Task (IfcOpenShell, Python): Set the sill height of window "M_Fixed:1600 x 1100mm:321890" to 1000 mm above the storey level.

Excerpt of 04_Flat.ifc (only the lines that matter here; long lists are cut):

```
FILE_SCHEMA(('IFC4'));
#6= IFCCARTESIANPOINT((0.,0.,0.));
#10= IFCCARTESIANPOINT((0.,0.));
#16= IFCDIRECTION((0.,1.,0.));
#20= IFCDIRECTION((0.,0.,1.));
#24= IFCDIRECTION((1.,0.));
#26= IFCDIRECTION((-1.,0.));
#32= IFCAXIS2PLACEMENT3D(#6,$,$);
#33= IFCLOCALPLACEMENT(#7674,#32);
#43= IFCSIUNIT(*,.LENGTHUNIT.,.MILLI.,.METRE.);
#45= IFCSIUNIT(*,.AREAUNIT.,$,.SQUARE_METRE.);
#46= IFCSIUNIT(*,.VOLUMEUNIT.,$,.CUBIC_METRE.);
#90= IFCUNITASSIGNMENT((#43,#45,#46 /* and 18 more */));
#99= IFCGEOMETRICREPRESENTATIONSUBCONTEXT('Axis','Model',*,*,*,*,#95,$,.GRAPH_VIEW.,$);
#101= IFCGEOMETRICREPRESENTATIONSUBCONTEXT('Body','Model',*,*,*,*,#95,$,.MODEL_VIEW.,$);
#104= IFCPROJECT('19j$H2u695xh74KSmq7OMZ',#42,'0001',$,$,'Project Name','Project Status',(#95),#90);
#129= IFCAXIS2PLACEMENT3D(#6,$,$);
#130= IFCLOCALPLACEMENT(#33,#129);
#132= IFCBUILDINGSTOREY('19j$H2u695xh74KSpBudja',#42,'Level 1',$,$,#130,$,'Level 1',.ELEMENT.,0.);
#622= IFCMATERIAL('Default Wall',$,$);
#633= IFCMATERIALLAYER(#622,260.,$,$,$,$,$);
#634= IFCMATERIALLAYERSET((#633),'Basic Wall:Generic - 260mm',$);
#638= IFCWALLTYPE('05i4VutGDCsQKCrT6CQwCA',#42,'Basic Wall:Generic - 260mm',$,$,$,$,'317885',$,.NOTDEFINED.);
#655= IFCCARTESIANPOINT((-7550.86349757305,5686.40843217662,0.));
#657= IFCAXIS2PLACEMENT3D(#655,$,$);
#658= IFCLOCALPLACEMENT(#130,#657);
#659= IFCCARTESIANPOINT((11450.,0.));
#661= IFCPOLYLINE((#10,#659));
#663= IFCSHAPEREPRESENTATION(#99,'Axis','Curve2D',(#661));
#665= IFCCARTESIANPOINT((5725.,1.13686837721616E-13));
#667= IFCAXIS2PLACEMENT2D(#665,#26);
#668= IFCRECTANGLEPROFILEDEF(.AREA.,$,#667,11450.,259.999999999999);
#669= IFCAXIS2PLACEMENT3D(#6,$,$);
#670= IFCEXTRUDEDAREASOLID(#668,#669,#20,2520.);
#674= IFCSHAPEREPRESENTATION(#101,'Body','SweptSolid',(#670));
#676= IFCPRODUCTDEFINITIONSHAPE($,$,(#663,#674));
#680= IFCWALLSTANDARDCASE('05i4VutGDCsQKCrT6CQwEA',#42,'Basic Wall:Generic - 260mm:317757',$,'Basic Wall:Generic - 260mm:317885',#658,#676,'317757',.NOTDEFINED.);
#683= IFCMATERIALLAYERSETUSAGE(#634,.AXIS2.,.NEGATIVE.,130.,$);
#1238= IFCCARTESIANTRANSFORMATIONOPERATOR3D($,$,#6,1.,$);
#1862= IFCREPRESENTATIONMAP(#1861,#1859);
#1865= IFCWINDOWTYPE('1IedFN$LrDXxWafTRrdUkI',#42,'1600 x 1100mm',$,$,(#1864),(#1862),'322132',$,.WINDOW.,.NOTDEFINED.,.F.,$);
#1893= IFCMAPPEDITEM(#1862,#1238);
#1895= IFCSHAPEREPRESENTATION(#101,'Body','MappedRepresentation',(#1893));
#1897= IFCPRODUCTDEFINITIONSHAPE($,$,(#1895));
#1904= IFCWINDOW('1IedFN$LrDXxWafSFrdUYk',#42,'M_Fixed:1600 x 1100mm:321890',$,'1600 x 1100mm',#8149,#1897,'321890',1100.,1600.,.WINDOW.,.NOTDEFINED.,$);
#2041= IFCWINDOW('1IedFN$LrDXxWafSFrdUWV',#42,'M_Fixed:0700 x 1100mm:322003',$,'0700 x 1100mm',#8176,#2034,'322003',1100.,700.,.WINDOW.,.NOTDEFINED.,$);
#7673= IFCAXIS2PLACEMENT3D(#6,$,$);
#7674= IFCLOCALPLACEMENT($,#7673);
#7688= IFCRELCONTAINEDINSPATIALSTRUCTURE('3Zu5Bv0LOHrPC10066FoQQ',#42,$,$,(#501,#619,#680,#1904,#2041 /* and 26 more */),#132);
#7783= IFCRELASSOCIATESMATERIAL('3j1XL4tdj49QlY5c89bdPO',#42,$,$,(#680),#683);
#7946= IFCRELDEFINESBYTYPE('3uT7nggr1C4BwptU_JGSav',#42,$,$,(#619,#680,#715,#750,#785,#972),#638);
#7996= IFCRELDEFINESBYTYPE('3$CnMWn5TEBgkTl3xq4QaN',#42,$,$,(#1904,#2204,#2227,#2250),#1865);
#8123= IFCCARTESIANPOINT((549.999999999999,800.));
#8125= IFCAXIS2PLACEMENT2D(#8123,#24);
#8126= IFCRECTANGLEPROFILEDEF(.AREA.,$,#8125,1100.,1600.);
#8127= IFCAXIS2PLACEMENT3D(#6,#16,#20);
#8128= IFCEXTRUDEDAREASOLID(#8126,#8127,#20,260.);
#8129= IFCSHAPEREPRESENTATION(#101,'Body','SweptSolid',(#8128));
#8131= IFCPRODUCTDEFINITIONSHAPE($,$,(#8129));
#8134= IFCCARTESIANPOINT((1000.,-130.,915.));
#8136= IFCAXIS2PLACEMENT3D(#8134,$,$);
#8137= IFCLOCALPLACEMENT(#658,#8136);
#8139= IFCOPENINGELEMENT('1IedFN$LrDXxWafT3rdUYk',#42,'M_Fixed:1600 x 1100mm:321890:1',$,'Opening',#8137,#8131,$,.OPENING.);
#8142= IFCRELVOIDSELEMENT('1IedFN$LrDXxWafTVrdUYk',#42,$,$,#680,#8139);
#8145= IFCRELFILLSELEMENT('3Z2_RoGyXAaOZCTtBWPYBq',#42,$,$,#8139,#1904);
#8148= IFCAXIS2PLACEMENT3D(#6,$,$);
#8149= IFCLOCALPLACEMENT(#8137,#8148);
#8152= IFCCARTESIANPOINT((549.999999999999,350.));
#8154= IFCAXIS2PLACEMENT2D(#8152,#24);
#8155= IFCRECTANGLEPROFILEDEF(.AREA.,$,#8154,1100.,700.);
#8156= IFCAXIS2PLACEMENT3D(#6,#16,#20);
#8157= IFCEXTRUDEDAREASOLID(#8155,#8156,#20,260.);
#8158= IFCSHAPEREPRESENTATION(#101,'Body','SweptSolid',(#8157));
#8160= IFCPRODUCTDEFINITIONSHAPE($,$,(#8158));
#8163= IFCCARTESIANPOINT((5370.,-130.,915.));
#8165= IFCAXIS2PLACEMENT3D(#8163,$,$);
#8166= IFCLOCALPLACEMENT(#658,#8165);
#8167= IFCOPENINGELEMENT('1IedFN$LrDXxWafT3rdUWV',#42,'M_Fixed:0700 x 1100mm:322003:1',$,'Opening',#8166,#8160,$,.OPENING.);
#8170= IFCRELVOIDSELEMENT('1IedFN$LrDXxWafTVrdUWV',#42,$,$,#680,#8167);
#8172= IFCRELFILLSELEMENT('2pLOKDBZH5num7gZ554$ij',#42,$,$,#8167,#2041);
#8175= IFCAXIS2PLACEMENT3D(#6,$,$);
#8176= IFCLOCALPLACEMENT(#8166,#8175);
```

```python
import numpy as np
import ifcopenshell
import ifcopenshell.api.geometry
import ifcopenshell.geom
import ifcopenshell.util.element
import ifcopenshell.util.placement
import ifcopenshell.util.shape
import ifcopenshell.util.unit

model = ifcopenshell.open("04_Flat.ifc")
unit_scale = ifcopenshell.util.unit.calculate_unit_scale(model)

window = model.by_guid("1IedFN$LrDXxWafSFrdUYk")
opening = window.FillsVoids[0].RelatingOpeningElement
storey = ifcopenshell.util.element.get_container(window, ifc_class="IfcBuildingStorey")
level = ifcopenshell.util.placement.get_local_placement(storey.ObjectPlacement)[2, 3]

# The opening's origin need not be at the sill, so measure its lowest point.
shape = ifcopenshell.geom.create_shape(ifcopenshell.geom.settings(), opening)
bottom = ifcopenshell.util.shape.get_shape_bottom_elevation(shape, shape.geometry) / unit_scale
dz = level + 1 / unit_scale - bottom

shift = np.array([0.0, 0.0, dz])
# The window is placed relative to its opening, so it follows when the opening moves.
matrix = ifcopenshell.util.placement.get_local_placement(opening.ObjectPlacement)
matrix[:3, 3] += shift
ifcopenshell.api.geometry.edit_object_placement(
    model, product=opening, matrix=matrix, is_si=False, should_transform_children=True
)

print(f"moved by {dz * unit_scale:+.3f} m")

model.write("04_Flat_v2.ifc")
```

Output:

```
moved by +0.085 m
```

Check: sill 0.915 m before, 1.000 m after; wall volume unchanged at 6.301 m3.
